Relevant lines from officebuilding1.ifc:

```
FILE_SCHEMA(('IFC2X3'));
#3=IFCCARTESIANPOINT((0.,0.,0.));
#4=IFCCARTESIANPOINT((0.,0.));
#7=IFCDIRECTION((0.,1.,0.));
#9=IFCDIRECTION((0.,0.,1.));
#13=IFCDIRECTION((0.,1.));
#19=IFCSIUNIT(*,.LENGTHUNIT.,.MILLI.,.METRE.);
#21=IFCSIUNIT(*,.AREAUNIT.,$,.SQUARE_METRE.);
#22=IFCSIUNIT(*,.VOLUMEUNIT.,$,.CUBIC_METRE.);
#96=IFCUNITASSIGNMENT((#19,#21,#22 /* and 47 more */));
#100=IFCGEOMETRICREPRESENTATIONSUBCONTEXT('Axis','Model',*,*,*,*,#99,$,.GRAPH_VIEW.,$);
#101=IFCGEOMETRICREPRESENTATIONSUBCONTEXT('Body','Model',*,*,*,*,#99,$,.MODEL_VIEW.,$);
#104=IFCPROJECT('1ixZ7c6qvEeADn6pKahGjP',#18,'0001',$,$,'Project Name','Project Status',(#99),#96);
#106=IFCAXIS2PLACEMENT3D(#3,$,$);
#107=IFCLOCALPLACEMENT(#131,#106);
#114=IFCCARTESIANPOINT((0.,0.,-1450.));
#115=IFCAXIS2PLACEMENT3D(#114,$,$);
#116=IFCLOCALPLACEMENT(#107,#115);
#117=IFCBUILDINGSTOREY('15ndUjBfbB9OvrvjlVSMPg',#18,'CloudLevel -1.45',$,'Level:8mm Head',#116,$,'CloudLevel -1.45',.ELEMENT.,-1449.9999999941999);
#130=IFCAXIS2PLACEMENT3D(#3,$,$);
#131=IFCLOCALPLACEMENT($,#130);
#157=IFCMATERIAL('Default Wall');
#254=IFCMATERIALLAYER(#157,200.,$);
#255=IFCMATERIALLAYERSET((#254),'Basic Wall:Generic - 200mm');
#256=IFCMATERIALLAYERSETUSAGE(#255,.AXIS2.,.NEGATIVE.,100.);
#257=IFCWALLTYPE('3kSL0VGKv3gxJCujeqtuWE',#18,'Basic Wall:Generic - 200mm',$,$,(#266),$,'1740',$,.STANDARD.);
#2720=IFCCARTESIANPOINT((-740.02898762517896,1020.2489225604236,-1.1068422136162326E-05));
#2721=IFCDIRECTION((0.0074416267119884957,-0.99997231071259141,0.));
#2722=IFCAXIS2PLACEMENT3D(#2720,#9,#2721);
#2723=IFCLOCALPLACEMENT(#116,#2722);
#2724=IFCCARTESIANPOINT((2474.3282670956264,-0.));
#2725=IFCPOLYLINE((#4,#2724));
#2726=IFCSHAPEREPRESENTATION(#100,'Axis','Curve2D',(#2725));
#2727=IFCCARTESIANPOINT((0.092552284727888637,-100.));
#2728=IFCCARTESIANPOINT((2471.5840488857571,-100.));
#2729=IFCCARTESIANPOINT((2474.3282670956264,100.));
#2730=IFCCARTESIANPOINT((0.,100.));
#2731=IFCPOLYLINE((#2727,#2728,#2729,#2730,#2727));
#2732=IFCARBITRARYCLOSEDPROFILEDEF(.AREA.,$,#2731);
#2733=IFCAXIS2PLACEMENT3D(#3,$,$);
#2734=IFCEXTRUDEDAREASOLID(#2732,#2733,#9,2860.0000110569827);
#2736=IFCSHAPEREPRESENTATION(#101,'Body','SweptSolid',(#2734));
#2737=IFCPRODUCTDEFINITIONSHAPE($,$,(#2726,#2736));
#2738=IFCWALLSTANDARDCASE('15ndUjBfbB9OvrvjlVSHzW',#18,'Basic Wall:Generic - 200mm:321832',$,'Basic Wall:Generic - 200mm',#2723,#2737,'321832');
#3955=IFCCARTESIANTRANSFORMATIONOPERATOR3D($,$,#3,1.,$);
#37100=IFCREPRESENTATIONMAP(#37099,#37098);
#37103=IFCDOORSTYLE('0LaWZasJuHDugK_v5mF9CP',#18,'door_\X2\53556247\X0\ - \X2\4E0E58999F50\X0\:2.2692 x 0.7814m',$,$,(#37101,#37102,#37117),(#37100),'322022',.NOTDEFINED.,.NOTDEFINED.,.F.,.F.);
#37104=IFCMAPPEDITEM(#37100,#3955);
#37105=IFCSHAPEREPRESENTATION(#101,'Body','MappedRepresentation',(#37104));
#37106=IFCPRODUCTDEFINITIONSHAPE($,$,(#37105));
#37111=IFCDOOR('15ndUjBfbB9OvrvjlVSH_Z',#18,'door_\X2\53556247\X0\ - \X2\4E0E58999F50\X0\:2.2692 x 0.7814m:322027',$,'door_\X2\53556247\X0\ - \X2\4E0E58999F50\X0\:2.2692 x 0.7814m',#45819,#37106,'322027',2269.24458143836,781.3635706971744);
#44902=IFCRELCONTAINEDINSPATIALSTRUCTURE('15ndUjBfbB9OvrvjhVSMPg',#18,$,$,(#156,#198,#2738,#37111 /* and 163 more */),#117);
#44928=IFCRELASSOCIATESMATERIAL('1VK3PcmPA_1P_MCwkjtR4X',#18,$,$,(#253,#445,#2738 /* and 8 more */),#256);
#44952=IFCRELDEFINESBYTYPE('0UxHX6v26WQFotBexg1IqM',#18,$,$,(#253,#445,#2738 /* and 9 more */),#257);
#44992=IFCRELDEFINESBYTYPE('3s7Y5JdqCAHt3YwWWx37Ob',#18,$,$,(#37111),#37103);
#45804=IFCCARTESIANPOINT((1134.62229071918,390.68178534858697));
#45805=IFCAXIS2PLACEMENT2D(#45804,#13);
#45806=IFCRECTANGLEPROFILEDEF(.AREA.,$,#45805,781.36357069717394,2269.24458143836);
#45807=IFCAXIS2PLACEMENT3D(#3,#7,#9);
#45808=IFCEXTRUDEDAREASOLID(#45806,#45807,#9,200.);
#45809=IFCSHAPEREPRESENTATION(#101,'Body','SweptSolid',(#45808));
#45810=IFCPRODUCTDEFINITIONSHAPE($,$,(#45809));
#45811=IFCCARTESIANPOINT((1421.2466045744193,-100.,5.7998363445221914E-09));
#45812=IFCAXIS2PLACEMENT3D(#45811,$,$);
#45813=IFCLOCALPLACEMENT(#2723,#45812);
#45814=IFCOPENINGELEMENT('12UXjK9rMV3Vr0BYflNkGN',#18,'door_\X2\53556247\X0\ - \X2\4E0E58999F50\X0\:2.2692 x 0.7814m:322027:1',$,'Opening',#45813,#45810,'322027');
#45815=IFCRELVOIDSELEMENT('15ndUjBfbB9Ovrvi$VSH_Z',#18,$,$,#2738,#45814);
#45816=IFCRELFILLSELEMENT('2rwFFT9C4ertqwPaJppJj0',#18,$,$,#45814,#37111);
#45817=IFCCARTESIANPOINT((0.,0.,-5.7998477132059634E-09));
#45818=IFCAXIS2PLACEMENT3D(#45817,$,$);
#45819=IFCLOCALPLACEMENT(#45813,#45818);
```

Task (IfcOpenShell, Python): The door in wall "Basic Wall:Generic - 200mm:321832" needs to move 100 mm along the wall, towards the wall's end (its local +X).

```python
import ifcopenshell
import ifcopenshell.api.geometry
import ifcopenshell.util.placement

model = ifcopenshell.open("officebuilding1.ifc")

door = model.by_guid("15ndUjBfbB9OvrvjlVSH_Z")
opening = door.FillsVoids[0].RelatingOpeningElement
wall = opening.VoidsElements[0].RelatingBuildingElement

wall_matrix = ifcopenshell.util.placement.get_local_placement(wall.ObjectPlacement)
shift = wall_matrix[:3, 0] * 100.0
before = ifcopenshell.util.placement.get_local_placement(door.ObjectPlacement)[:3, 3].copy()

# The door is placed relative to its opening, so it follows when the opening moves.
matrix = ifcopenshell.util.placement.get_local_placement(opening.ObjectPlacement)
matrix[:3, 3] += shift
ifcopenshell.api.geometry.edit_object_placement(
    model, product=opening, matrix=matrix, is_si=False, should_transform_children=True
)

after = ifcopenshell.util.placement.get_local_placement(door.ObjectPlacement)[:3, 3]
print("door moved by", (after - before).round(3) + 0.0)

model.write("officebuilding1_v2.ifc")
```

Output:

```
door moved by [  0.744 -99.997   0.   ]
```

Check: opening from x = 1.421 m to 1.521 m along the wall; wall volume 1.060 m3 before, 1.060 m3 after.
